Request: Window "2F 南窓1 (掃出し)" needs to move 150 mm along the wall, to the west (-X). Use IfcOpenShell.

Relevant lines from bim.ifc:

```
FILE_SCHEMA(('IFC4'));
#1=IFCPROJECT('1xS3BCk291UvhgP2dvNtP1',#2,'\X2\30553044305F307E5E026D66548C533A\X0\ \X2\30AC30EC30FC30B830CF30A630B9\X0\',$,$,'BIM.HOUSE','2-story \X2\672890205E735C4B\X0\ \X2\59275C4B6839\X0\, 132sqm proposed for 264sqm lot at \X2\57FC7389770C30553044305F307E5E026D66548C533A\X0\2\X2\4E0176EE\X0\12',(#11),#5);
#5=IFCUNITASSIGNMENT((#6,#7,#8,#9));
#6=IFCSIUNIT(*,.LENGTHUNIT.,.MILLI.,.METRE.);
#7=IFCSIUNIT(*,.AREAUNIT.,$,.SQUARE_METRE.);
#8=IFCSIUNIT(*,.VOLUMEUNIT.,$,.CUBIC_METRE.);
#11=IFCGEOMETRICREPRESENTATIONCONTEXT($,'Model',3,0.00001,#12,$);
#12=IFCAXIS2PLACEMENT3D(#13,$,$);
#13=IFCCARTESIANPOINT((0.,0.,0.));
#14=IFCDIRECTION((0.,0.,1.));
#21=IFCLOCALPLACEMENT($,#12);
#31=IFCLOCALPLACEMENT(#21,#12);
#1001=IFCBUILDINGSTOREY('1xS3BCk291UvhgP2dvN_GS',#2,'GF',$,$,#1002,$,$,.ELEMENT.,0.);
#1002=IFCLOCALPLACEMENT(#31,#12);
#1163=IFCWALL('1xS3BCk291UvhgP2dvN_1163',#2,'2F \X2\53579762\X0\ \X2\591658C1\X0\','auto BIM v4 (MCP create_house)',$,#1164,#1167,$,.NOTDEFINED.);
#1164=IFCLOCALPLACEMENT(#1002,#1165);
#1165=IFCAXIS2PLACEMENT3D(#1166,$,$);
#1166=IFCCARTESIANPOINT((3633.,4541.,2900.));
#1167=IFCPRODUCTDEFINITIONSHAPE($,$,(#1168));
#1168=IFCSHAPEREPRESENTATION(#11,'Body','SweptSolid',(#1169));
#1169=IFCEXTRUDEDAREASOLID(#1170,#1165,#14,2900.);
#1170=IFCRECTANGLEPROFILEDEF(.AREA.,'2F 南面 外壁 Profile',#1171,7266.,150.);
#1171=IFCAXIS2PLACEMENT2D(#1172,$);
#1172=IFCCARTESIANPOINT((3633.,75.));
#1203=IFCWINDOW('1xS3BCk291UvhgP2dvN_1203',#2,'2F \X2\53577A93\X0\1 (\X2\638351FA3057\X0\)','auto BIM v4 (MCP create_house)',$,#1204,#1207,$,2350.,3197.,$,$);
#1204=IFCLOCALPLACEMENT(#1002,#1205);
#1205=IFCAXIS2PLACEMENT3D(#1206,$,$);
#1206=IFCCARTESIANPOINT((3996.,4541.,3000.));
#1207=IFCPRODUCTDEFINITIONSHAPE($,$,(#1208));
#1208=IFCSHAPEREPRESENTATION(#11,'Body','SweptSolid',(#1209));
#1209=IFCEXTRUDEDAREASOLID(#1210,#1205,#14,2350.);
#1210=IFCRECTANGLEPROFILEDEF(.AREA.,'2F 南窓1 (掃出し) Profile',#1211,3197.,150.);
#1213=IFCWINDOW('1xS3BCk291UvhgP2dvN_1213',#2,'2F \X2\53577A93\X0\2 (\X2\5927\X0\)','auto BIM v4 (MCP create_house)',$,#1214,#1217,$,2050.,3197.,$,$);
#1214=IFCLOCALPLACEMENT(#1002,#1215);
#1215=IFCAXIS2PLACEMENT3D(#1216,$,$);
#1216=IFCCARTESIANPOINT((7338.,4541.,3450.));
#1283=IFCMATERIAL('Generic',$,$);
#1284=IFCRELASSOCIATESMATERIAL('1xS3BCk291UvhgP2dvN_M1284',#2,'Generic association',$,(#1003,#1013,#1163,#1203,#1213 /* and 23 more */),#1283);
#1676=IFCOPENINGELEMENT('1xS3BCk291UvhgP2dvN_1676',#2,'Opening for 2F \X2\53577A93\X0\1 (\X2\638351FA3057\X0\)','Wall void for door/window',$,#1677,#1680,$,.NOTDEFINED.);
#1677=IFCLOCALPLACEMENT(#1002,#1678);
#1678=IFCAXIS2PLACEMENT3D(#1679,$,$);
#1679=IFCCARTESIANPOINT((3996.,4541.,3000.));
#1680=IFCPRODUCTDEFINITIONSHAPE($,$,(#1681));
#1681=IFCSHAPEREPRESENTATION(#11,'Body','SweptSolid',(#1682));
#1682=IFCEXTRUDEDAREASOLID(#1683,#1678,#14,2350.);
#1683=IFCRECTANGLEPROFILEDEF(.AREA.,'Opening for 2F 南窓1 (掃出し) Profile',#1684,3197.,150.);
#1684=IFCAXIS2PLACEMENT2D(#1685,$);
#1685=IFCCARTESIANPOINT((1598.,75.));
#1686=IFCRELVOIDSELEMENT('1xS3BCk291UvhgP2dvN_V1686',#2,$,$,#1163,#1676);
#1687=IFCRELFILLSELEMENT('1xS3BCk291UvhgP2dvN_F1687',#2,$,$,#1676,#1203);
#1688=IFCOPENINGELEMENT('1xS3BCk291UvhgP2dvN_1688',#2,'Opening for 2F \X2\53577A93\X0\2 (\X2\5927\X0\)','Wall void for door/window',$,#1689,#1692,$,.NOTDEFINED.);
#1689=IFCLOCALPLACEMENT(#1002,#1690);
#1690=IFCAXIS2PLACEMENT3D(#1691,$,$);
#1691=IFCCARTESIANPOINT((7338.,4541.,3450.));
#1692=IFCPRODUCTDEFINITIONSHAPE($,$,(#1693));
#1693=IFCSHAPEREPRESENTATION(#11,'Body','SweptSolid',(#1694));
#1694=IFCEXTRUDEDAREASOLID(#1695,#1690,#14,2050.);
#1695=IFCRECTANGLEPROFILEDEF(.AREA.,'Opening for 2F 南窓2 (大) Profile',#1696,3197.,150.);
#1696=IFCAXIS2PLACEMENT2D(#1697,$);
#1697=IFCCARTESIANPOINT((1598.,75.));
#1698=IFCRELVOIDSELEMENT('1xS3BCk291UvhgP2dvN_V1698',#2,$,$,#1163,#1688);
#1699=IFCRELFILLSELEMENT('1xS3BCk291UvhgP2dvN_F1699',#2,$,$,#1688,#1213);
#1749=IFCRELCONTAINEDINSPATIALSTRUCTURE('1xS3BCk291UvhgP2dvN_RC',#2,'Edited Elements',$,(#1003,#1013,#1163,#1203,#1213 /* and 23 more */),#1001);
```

```python
import ifcopenshell
import ifcopenshell.api.geometry
import ifcopenshell.util.placement
import ifcopenshell.util.unit

model = ifcopenshell.open("bim.ifc")
unit_scale = ifcopenshell.util.unit.calculate_unit_scale(model)

window = model.by_id(1203)
opening = window.FillsVoids[0].RelatingOpeningElement
wall = opening.VoidsElements[0].RelatingBuildingElement

wall_matrix = ifcopenshell.util.placement.get_local_placement(wall.ObjectPlacement)
shift = wall_matrix[:3, 0] * -0.15 / unit_scale
before = ifcopenshell.util.placement.get_local_placement(window.ObjectPlacement)[:3, 3].copy()

# The window is not placed relative to its opening, so move both.
for product in (opening, window):
    matrix = ifcopenshell.util.placement.get_local_placement(product.ObjectPlacement)
    matrix[:3, 3] += shift
    ifcopenshell.api.geometry.edit_object_placement(model, product=product, matrix=matrix, is_si=False)

after = ifcopenshell.util.placement.get_local_placement(window.ObjectPlacement)[:3, 3]
print("window moved by", (after - before).round(3) + 0.0)

model.write("bim-out.ifc")
```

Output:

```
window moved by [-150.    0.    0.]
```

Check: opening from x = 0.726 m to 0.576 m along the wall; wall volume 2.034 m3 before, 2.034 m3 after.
